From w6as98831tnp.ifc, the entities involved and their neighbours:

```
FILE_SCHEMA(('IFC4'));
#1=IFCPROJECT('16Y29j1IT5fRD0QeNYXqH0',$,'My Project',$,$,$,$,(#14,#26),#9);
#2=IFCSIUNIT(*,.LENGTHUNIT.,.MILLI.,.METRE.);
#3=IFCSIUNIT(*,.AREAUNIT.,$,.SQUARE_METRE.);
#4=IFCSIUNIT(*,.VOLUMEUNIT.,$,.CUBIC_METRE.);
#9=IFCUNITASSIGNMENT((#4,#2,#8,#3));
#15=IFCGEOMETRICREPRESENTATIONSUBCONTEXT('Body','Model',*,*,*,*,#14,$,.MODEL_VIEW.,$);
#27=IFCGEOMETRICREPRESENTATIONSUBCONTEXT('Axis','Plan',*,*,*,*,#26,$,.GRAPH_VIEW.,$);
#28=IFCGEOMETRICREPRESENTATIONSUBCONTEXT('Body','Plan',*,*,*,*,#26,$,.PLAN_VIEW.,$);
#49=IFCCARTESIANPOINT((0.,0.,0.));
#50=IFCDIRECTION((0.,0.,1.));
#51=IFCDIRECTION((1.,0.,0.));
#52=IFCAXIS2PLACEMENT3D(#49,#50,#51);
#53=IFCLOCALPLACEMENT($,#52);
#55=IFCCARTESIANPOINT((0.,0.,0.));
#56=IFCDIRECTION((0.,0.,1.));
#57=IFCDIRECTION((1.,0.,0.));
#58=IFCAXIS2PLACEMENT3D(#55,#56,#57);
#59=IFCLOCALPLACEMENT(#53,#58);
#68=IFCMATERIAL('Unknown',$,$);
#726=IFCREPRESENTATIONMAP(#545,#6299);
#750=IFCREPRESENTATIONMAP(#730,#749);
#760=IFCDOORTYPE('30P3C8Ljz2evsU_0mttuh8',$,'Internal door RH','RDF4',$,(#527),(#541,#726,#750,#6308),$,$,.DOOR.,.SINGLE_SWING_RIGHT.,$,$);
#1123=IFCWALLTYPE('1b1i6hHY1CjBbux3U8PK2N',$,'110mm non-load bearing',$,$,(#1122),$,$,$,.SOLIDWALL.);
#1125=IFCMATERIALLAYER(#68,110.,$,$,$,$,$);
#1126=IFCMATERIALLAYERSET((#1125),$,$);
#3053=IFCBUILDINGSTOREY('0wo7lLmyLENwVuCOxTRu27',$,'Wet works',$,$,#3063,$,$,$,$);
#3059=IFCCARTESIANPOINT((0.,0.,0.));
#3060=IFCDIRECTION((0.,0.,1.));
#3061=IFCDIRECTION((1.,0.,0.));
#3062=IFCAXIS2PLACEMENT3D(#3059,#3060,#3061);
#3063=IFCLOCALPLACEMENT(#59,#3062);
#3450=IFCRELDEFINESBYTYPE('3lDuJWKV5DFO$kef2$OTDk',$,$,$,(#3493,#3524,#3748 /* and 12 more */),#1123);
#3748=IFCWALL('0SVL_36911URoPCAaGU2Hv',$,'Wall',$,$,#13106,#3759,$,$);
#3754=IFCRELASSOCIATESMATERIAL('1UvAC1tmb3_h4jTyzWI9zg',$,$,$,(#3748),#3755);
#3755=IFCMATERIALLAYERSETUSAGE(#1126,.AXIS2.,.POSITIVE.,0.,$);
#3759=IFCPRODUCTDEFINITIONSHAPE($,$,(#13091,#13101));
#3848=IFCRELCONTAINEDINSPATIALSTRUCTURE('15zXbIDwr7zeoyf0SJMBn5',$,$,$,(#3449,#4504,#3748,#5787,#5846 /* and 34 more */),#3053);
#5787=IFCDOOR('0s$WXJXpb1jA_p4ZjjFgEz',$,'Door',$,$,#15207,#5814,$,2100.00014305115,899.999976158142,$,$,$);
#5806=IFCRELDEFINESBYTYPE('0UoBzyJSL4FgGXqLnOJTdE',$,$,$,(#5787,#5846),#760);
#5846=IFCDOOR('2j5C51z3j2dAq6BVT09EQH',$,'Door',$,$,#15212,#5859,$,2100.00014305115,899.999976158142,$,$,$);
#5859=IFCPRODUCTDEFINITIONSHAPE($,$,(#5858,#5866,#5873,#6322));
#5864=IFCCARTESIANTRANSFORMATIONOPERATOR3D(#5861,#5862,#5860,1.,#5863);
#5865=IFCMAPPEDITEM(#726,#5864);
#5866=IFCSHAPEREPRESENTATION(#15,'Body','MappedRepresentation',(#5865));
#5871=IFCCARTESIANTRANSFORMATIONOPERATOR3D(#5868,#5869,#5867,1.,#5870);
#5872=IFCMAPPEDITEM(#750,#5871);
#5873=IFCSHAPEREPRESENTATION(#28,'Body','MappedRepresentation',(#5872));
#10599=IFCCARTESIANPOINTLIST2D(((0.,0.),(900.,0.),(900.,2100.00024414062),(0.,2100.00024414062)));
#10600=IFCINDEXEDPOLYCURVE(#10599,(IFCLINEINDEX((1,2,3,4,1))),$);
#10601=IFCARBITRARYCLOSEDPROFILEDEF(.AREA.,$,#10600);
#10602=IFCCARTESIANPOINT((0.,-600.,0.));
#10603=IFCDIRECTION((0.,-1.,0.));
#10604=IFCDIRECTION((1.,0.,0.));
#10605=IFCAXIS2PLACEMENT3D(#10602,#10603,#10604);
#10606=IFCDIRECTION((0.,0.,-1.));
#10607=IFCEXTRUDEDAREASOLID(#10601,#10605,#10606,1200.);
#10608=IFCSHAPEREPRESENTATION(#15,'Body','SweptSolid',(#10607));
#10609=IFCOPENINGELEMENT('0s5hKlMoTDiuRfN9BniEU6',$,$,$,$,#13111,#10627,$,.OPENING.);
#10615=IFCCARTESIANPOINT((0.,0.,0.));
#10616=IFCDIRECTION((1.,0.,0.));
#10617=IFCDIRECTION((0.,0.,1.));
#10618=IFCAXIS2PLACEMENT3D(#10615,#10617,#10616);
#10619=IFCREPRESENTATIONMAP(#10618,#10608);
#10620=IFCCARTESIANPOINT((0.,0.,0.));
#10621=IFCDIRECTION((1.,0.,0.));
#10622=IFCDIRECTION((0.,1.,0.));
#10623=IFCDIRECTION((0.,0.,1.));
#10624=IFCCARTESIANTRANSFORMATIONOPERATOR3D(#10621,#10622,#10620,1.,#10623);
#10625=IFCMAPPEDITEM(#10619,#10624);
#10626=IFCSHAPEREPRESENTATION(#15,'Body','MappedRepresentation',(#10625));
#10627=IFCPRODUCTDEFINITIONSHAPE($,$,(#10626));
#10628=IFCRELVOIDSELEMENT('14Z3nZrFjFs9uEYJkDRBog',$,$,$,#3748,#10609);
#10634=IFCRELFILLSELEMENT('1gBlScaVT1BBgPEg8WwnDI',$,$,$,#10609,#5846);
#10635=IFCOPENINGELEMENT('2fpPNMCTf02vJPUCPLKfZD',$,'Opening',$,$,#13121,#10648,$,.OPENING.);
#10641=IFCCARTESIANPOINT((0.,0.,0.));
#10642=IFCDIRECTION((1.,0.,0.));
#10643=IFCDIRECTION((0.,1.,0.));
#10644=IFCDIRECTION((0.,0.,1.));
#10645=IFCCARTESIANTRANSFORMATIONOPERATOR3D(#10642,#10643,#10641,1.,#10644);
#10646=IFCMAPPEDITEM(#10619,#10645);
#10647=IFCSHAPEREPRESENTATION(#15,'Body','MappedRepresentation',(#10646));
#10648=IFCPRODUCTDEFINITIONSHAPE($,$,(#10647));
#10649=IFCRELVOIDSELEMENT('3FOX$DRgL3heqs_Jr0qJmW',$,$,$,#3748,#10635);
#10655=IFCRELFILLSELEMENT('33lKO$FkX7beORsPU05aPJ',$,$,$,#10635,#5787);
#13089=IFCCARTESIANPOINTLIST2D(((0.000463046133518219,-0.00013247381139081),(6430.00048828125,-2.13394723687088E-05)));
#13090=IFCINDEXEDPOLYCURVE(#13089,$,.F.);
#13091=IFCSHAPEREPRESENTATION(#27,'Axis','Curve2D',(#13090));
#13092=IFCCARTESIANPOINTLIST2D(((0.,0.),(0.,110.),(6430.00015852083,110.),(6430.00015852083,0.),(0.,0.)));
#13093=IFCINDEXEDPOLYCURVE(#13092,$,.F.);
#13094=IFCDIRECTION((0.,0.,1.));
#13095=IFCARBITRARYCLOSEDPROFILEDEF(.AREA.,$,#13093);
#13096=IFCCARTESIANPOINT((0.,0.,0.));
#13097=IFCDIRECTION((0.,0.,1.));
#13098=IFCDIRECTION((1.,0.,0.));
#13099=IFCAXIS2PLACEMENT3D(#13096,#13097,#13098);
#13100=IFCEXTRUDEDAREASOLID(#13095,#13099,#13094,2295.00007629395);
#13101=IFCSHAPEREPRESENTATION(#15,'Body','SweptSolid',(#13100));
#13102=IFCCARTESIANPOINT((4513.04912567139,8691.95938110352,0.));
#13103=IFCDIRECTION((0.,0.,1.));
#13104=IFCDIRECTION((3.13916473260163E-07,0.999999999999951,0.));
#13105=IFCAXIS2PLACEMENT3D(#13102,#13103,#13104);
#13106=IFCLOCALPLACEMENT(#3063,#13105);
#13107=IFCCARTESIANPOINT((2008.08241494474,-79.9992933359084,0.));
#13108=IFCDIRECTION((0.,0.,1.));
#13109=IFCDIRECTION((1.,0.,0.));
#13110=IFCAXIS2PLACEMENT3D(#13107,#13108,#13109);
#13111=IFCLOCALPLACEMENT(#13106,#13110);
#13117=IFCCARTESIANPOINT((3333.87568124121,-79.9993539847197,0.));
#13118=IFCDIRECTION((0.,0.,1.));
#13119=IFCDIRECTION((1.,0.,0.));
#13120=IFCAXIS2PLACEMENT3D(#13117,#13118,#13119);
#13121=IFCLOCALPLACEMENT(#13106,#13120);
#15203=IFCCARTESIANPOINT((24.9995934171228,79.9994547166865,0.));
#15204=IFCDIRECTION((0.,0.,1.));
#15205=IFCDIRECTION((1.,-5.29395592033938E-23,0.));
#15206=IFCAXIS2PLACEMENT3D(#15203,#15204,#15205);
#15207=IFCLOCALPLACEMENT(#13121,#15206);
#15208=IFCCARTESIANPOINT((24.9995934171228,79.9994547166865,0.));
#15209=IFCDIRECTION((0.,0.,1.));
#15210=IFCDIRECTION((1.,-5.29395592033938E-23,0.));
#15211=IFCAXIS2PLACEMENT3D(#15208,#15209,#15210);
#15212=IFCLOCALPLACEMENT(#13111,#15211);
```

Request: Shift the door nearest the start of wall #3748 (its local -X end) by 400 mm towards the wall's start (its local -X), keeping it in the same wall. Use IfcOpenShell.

```python
import ifcopenshell
import ifcopenshell.api.geometry
import ifcopenshell.util.placement
import ifcopenshell.util.unit

model = ifcopenshell.open("w6as98831tnp.ifc")
unit_scale = ifcopenshell.util.unit.calculate_unit_scale(model)

door = model.by_guid("2j5C51z3j2dAq6BVT09EQH")
opening = door.FillsVoids[0].RelatingOpeningElement
wall = opening.VoidsElements[0].RelatingBuildingElement

wall_matrix = ifcopenshell.util.placement.get_local_placement(wall.ObjectPlacement)
shift = wall_matrix[:3, 0] * -0.4 / unit_scale
before = ifcopenshell.util.placement.get_local_placement(door.ObjectPlacement)[:3, 3].copy()

# The door is placed relative to its opening, so it follows when the opening moves.
matrix = ifcopenshell.util.placement.get_local_placement(opening.ObjectPlacement)
matrix[:3, 3] += shift
ifcopenshell.api.geometry.edit_object_placement(
    model, product=opening, matrix=matrix, is_si=False, should_transform_children=True
)

after = ifcopenshell.util.placement.get_local_placement(door.ObjectPlacement)[:3, 3]
print("door moved by", (after - before).round(3) + 0.0)

model.write("w6as98831tnp_edited.ifc")
```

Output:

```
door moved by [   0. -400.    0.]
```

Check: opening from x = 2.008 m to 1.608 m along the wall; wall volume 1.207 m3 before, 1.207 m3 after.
